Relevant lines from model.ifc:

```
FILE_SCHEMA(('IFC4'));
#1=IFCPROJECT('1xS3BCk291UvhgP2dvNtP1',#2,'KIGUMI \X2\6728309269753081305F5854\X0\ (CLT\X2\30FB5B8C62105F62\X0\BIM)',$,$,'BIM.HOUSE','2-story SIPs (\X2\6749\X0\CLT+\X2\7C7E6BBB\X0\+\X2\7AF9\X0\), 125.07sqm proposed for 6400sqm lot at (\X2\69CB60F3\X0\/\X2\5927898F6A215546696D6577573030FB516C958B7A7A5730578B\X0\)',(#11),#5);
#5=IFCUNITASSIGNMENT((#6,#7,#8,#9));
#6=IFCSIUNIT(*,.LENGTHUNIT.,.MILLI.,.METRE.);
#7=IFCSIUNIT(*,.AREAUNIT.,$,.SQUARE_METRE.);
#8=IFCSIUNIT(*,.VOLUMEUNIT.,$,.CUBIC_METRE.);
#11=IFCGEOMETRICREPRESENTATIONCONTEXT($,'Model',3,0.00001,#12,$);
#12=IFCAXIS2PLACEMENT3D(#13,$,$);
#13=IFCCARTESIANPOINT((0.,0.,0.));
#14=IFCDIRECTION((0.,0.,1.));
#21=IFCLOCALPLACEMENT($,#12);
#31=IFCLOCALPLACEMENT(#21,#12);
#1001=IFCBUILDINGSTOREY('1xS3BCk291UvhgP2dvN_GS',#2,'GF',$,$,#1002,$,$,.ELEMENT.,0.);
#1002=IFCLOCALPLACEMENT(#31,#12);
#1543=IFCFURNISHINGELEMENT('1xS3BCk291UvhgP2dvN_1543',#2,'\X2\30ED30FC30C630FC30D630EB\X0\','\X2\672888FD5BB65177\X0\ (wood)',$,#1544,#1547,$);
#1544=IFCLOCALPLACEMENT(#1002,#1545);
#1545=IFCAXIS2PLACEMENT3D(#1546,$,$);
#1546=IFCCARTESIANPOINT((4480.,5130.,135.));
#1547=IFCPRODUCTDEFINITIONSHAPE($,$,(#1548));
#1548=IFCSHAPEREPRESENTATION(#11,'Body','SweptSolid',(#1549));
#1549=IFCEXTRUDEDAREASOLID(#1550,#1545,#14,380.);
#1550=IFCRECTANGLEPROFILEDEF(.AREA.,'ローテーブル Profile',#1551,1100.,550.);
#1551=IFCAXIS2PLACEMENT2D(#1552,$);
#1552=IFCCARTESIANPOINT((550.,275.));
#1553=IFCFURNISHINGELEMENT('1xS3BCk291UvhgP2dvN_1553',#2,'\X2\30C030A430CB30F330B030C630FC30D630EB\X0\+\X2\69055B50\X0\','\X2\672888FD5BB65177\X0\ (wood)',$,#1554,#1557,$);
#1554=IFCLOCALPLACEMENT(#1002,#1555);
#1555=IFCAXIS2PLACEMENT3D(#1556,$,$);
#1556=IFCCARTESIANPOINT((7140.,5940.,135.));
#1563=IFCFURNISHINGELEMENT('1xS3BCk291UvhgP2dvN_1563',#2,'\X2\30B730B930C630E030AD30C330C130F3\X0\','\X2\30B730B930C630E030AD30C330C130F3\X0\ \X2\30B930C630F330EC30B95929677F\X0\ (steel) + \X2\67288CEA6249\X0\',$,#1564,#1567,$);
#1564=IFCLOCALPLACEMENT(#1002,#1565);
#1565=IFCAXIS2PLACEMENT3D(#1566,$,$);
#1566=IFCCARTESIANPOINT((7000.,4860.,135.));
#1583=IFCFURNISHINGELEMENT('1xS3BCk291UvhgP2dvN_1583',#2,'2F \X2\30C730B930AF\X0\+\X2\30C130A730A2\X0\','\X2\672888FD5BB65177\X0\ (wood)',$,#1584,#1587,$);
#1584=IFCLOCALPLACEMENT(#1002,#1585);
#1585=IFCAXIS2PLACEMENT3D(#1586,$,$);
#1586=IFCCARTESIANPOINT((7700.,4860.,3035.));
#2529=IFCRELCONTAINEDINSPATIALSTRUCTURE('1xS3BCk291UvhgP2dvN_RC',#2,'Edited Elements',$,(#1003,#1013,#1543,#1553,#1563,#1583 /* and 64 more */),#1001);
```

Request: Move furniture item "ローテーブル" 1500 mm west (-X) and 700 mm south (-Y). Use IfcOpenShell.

```python
import ifcopenshell
import ifcopenshell.api.geometry
import ifcopenshell.util.placement
import ifcopenshell.util.unit

model = ifcopenshell.open("model.ifc")
unit_scale = ifcopenshell.util.unit.calculate_unit_scale(model)

item = model.by_guid("1xS3BCk291UvhgP2dvN_1543")
matrix = ifcopenshell.util.placement.get_local_placement(item.ObjectPlacement)
matrix[0, 3] -= 1.5 / unit_scale
matrix[1, 3] -= 0.7 / unit_scale
ifcopenshell.api.geometry.edit_object_placement(model, product=item, matrix=matrix, is_si=False)

print(ifcopenshell.util.placement.get_local_placement(item.ObjectPlacement).round(3) + 0.0)

model.write("model_updated.ifc")
```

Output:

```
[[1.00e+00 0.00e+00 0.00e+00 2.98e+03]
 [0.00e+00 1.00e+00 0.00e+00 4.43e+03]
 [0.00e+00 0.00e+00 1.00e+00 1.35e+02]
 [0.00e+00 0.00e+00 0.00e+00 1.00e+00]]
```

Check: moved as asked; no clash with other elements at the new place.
